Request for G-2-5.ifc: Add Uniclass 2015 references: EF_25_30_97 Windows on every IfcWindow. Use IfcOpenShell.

First a look at what the model holds.

```python
import ifcopenshell

model = ifcopenshell.open("G-2-5.ifc")
print(model.schema)
print("classifications:", [c.Name for c in model.by_type("IfcClassification")])
for ifc_class in ("IfcDoor", "IfcRoof", "IfcStair", "IfcWall", "IfcWindow"):
    print(ifc_class, len(model.by_type(ifc_class)))
```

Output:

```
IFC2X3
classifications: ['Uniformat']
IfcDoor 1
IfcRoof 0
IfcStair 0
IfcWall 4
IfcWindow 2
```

```python
import ifcopenshell
import ifcopenshell.api.classification

model = ifcopenshell.open("G-2-5.ifc")

# IFC2X3 requires Source and Edition and has no link from the project to the system.
system = model.create_entity("IfcClassification", Source="NBS", Edition="2015", Name="Uniclass 2015")

codes = {
    "IfcWindow": ("EF_25_30_97", "Windows"),
}
for ifc_class, (code, name) in codes.items():
    products = model.by_type(ifc_class)
    ifcopenshell.api.classification.add_reference(
        model, products=products, classification=system, identification=code, name=name
    )
    print(code, len(products))

model.write("G-2-5-out.ifc")
```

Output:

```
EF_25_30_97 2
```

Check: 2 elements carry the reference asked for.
